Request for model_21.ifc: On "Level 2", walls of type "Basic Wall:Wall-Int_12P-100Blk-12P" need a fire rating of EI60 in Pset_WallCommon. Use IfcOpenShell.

First a look at what the model holds.

```python
import ifcopenshell
import ifcopenshell.util.element

model = ifcopenshell.open("model_21.ifc")
print(model.schema)
storey = next(s for s in model.by_type("IfcBuildingStorey") if s.Name == "Level 2")
walls = [e for e in ifcopenshell.util.element.get_decomposition(storey) if e.is_a("IfcWall")]
seen = {}
for e in walls:
    element_type = ifcopenshell.util.element.get_type(e)
    key = (element_type.Name if element_type != e and element_type else None, ifcopenshell.util.element.get_pset(e, "Pset_WallCommon", "FireRating"))
    seen[key] = seen.get(key, 0) + 1
for (name, value), count in sorted(seen.items(), key=str):
    print(count, "x", name, "|", value)
```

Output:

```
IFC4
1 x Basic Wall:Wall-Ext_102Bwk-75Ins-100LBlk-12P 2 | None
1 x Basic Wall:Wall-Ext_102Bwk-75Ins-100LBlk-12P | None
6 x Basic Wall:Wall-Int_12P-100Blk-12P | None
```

```python
import ifcopenshell
import ifcopenshell.api.pset
import ifcopenshell.util.element

model = ifcopenshell.open("model_21.ifc")

storey = next(s for s in model.by_type("IfcBuildingStorey") if s.Name == "Level 2")
walls = [e for e in ifcopenshell.util.element.get_decomposition(storey) if e.is_a("IfcWall")]

count = 0
for e in walls:
    element_type = ifcopenshell.util.element.get_type(e)
    if element_type in (None, e) or element_type.Name != "Basic Wall:Wall-Int_12P-100Blk-12P":
        continue
    # add_pset returns the element's existing set when there is one.
    pset = ifcopenshell.api.pset.add_pset(model, product=e, name="Pset_WallCommon")
    ifcopenshell.api.pset.edit_pset(model, pset=pset, properties={"FireRating": "EI60"})
    count += 1

print(count, "walls updated")

model.write("model_21_updated.ifc")
```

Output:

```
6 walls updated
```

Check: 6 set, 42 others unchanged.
